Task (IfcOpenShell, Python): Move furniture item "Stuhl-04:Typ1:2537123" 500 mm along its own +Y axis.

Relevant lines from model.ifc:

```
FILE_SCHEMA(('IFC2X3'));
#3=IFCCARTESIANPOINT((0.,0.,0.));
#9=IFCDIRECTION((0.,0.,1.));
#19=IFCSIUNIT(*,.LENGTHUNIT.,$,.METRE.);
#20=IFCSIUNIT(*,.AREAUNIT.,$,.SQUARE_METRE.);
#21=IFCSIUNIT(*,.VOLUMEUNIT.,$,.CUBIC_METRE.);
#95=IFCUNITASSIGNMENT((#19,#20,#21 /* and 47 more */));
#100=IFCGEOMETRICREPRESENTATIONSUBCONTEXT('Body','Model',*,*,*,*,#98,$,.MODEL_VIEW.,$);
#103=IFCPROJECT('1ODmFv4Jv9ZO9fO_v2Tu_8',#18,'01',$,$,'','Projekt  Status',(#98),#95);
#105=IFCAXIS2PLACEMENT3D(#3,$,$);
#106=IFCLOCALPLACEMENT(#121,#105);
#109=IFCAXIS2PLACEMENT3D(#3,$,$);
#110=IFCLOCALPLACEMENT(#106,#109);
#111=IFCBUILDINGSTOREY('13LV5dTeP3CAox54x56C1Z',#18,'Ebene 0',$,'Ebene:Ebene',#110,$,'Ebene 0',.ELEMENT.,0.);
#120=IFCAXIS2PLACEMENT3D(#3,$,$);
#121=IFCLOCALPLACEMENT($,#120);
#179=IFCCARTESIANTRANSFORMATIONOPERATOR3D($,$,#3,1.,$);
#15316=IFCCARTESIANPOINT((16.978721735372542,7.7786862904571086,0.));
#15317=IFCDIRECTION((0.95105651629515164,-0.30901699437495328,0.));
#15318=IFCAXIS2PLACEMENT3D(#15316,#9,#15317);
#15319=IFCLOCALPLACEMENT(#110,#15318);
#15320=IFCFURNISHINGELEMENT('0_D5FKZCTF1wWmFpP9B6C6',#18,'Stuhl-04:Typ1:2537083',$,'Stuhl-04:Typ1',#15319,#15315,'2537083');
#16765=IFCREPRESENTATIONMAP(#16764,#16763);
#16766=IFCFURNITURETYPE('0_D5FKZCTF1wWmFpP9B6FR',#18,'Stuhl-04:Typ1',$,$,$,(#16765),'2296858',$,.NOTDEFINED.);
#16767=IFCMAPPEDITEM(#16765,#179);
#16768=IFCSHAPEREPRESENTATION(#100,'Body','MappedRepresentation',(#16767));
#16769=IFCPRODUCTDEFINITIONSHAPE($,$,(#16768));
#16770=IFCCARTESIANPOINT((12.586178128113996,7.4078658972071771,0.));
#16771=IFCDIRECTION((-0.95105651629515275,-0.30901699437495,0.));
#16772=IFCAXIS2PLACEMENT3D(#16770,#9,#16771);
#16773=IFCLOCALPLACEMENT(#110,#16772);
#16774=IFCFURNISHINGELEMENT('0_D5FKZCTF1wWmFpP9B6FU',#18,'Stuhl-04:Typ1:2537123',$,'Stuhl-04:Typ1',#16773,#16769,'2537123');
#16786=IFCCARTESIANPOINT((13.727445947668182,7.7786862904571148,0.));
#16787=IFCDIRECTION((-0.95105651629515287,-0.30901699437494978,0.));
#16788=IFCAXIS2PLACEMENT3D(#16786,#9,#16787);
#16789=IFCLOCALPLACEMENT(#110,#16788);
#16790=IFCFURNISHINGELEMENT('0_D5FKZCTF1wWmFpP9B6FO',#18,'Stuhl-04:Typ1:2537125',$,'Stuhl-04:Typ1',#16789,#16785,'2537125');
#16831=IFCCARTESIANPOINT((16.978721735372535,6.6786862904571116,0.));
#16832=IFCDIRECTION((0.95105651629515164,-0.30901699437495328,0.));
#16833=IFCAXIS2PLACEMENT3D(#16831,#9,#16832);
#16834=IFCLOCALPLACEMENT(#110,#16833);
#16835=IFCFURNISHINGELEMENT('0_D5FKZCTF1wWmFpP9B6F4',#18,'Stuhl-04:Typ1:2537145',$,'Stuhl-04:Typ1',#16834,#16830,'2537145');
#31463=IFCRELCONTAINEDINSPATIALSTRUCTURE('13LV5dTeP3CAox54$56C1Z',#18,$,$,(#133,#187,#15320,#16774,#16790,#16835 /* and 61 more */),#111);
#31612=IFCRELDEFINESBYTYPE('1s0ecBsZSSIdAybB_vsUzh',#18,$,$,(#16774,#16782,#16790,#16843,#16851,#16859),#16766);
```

```python
import ifcopenshell
import ifcopenshell.api.geometry
import ifcopenshell.util.placement
import ifcopenshell.util.unit

model = ifcopenshell.open("model.ifc")
unit_scale = ifcopenshell.util.unit.calculate_unit_scale(model)

item = model.by_guid("0_D5FKZCTF1wWmFpP9B6FU")
matrix = ifcopenshell.util.placement.get_local_placement(item.ObjectPlacement)
matrix[:3, 3] += matrix[:3, 1] * 0.5 / unit_scale
ifcopenshell.api.geometry.edit_object_placement(model, product=item, matrix=matrix, is_si=False)

print(ifcopenshell.util.placement.get_local_placement(item.ObjectPlacement).round(3) + 0.0)

model.write("model_v2.ifc")
```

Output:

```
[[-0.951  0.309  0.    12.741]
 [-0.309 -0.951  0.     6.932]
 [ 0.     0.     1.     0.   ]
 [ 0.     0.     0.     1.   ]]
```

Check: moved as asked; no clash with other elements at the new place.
